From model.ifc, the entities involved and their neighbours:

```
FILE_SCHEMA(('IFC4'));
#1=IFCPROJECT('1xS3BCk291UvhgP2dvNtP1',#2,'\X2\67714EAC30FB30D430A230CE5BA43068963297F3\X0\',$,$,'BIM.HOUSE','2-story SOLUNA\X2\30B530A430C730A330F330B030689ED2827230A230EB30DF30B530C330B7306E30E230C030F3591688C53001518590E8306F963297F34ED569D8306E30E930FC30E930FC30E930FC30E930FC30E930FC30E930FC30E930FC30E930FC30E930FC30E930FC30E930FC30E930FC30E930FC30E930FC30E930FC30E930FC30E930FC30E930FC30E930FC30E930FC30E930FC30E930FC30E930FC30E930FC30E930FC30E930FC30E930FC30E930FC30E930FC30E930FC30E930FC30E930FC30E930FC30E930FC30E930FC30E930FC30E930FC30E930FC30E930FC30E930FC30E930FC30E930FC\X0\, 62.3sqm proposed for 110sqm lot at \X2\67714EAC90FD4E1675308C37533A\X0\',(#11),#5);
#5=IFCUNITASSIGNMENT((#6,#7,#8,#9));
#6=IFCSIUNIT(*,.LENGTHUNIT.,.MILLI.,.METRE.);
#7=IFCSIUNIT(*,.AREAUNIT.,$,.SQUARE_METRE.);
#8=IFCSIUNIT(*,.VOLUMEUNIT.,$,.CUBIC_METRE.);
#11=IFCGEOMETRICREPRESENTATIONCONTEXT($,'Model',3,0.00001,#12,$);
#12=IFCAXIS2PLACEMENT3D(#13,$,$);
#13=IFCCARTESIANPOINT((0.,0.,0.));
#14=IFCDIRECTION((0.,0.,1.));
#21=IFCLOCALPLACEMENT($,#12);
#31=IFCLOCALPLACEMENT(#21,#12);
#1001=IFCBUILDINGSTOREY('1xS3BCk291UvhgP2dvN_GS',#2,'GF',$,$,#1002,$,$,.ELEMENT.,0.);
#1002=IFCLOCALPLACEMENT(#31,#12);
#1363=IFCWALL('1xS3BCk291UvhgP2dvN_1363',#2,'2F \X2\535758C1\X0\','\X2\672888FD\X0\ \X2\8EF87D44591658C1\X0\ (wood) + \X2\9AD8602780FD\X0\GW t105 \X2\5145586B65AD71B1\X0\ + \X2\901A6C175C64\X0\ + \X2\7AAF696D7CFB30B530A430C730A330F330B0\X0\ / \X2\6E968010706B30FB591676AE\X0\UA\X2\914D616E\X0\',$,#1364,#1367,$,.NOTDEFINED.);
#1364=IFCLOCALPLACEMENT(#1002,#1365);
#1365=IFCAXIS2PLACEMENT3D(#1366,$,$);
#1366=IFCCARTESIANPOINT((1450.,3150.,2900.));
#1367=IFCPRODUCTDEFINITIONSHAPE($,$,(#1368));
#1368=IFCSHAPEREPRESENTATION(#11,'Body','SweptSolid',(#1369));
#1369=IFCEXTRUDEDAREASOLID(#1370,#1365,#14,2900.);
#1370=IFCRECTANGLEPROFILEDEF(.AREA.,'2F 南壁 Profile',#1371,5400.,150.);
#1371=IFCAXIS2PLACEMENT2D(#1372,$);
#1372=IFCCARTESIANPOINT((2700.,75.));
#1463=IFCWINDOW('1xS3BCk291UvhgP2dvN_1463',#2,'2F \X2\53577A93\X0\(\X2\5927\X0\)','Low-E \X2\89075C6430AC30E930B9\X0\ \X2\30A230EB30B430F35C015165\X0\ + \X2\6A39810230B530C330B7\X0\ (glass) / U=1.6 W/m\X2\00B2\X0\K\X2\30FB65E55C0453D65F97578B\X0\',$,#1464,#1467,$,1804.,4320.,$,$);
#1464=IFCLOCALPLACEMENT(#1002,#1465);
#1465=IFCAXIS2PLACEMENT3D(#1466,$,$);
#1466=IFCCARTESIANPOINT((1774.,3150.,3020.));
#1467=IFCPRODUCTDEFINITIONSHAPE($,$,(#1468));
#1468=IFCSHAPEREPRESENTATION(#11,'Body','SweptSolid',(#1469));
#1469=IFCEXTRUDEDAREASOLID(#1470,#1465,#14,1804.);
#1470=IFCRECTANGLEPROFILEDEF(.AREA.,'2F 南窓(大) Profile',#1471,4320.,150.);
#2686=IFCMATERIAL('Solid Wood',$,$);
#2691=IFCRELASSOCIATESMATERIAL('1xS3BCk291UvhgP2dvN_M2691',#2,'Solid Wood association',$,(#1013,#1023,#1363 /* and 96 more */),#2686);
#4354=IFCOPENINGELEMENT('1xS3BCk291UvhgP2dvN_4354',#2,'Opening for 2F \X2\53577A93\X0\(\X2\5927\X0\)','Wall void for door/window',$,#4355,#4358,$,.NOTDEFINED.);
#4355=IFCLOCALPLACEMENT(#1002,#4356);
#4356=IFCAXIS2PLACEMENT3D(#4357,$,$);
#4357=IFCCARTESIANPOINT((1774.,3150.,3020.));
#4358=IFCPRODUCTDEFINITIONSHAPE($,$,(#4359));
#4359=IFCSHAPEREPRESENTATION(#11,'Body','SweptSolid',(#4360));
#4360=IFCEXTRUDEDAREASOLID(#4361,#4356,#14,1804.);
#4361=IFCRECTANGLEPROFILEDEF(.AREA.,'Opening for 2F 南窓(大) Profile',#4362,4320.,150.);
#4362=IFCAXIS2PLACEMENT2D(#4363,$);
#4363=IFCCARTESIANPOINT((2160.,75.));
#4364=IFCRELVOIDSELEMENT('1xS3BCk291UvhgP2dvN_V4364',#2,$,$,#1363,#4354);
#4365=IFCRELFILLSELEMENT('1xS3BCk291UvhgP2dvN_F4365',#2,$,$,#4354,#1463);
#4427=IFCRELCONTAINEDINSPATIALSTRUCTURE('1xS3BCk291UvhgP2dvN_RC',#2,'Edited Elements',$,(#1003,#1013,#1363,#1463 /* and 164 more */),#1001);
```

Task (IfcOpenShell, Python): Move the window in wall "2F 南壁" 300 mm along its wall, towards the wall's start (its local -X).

```python
import ifcopenshell
import ifcopenshell.api.geometry
import ifcopenshell.util.placement

model = ifcopenshell.open("model.ifc")

window = model.by_guid("1xS3BCk291UvhgP2dvN_1463")
opening = window.FillsVoids[0].RelatingOpeningElement
wall = opening.VoidsElements[0].RelatingBuildingElement

wall_matrix = ifcopenshell.util.placement.get_local_placement(wall.ObjectPlacement)
shift = wall_matrix[:3, 0] * -300.0
before = ifcopenshell.util.placement.get_local_placement(window.ObjectPlacement)[:3, 3].copy()

# The window is not placed relative to its opening, so move both.
for product in (opening, window):
    matrix = ifcopenshell.util.placement.get_local_placement(product.ObjectPlacement)
    matrix[:3, 3] += shift
    ifcopenshell.api.geometry.edit_object_placement(model, product=product, matrix=matrix, is_si=False)

after = ifcopenshell.util.placement.get_local_placement(window.ObjectPlacement)[:3, 3]
print("window moved by", (after - before).round(3) + 0.0)

model.write("model-out.ifc")
```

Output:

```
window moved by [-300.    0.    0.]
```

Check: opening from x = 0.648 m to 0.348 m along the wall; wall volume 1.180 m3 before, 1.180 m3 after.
